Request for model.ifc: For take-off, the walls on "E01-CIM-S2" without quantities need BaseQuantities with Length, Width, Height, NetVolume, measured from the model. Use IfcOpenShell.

First a look at what the model holds.

```python
import ifcopenshell
import ifcopenshell.util.element
import ifcopenshell.util.unit

model = ifcopenshell.open("model.ifc")
print(model.schema)
for unit_type in ("LENGTHUNIT", "AREAUNIT", "VOLUMEUNIT"):
    print(unit_type, ifcopenshell.util.unit.calculate_unit_scale(model, unit_type))
storey = next(s for s in model.by_type("IfcBuildingStorey") if s.Name == "E01-CIM-S2")
walls = [e for e in ifcopenshell.util.element.get_decomposition(storey) if e.is_a("IfcWall")]
for e in sorted(walls, key=lambda e: e.id()):
    print(e.id(), e.is_a(), e.Name, list(ifcopenshell.util.element.get_psets(e, qtos_only=True)), sep=" | ")
```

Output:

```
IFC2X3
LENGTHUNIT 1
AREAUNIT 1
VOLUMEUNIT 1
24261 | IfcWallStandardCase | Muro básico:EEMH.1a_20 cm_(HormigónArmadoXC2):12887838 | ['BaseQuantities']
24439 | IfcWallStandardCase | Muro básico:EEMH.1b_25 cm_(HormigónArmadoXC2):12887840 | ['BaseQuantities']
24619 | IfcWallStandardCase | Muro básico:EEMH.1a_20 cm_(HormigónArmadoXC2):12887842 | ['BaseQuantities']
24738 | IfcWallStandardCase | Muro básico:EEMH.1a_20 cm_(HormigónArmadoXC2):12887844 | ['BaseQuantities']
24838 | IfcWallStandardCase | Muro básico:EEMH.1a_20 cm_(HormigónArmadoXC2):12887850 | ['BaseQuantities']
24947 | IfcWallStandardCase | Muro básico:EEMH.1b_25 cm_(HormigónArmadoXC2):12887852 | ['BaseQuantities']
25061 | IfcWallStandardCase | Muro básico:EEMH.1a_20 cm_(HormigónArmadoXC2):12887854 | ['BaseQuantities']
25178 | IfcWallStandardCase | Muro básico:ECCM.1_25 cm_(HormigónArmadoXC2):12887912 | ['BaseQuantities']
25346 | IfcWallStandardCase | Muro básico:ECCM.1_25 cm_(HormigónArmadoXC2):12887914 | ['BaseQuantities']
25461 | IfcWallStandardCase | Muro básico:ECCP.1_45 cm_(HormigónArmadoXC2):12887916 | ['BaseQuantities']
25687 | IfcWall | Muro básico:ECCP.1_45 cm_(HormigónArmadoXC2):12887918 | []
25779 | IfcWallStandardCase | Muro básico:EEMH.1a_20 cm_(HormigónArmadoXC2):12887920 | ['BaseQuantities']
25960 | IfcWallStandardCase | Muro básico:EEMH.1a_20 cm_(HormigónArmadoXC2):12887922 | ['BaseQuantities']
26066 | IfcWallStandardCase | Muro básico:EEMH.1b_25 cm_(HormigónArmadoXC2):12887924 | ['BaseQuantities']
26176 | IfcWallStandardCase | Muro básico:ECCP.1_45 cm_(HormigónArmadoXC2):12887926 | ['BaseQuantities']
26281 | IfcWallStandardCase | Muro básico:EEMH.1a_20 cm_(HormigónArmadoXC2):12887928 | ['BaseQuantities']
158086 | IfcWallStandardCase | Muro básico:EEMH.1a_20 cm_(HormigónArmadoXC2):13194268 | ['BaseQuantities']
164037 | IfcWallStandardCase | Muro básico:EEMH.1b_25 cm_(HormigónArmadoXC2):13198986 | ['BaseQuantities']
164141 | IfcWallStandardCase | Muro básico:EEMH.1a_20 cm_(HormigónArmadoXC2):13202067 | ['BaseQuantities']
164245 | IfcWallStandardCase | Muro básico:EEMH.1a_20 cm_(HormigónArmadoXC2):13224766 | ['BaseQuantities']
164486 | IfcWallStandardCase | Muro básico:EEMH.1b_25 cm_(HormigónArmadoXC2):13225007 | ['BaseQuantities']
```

```python
import ifcopenshell
import ifcopenshell.api.pset
import ifcopenshell.geom
import ifcopenshell.util.element
import ifcopenshell.util.shape
import ifcopenshell.util.unit

model = ifcopenshell.open("model.ifc")
unit_scale = ifcopenshell.util.unit.calculate_unit_scale(model)
volume_scale = ifcopenshell.util.unit.calculate_unit_scale(model, "VOLUMEUNIT")
settings = ifcopenshell.geom.settings()

storey = next(s for s in model.by_type("IfcBuildingStorey") if s.Name == "E01-CIM-S2")
walls = [e for e in ifcopenshell.util.element.get_decomposition(storey) if e.is_a("IfcWall")]

for e in sorted(walls, key=lambda e: e.id()):
    if ifcopenshell.util.element.get_psets(e, qtos_only=True, should_inherit=False):
        continue
    # Geometry comes back in metres, in the element's own axes.
    shape = ifcopenshell.geom.create_shape(settings, e)
    values = {
        "Length": ifcopenshell.util.shape.get_x(shape.geometry) / unit_scale,
        "Width": ifcopenshell.util.shape.get_y(shape.geometry) / unit_scale,
        "Height": ifcopenshell.util.shape.get_z(shape.geometry) / unit_scale,
        "NetVolume": ifcopenshell.util.shape.get_volume(shape.geometry) / volume_scale,
    }
    qto = ifcopenshell.api.pset.add_qto(model, product=e, name="BaseQuantities")
    ifcopenshell.api.pset.edit_qto(model, qto=qto, properties=values)
    print(e.id(), {k: round(v, 3) for k, v in values.items()})

model.write("model_v2.ifc")
```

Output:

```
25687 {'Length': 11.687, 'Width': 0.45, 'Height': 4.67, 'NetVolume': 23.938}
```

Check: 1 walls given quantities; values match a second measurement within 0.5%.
